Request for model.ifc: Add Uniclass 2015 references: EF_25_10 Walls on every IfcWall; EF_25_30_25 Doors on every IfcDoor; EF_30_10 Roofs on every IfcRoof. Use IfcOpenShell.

First a look at what the model holds.

```python
import ifcopenshell

model = ifcopenshell.open("model.ifc")
print(model.schema)
print("classifications:", [c.Name for c in model.by_type("IfcClassification")])
for ifc_class in ("IfcDoor", "IfcRoof", "IfcStair", "IfcWall", "IfcWindow"):
    print(ifc_class, len(model.by_type(ifc_class)))
```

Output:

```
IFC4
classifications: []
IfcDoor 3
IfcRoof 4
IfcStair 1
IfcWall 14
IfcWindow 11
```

```python
import ifcopenshell
import ifcopenshell.api.classification

model = ifcopenshell.open("model.ifc")

system = ifcopenshell.api.classification.add_classification(model, classification="Uniclass 2015")

codes = {
    "IfcWall": ("EF_25_10", "Walls"),
    "IfcDoor": ("EF_25_30_25", "Doors"),
    "IfcRoof": ("EF_30_10", "Roofs"),
}
for ifc_class, (code, name) in codes.items():
    products = model.by_type(ifc_class)
    ifcopenshell.api.classification.add_reference(
        model, products=products, classification=system, identification=code, name=name
    )
    print(code, len(products))

model.write("model-out.ifc")
```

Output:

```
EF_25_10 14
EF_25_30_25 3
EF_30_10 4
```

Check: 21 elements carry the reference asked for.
